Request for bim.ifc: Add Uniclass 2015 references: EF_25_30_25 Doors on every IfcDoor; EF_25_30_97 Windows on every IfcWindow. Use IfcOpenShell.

First a look at what the model holds.

```python
import ifcopenshell

model = ifcopenshell.open("bim.ifc")
print(model.schema)
print("classifications:", [c.Name for c in model.by_type("IfcClassification")])
for ifc_class in ("IfcDoor", "IfcRoof", "IfcStair", "IfcWall", "IfcWindow"):
    print(ifc_class, len(model.by_type(ifc_class)))
```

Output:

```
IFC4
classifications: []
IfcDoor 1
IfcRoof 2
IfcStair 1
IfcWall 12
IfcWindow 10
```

```python
import ifcopenshell
import ifcopenshell.api.classification

model = ifcopenshell.open("bim.ifc")

system = ifcopenshell.api.classification.add_classification(model, classification="Uniclass 2015")

codes = {
    "IfcDoor": ("EF_25_30_25", "Doors"),
    "IfcWindow": ("EF_25_30_97", "Windows"),
}
for ifc_class, (code, name) in codes.items():
    products = model.by_type(ifc_class)
    ifcopenshell.api.classification.add_reference(
        model, products=products, classification=system, identification=code, name=name
    )
    print(code, len(products))

model.write("bim-out.ifc")
```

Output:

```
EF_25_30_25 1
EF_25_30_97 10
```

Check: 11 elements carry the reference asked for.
